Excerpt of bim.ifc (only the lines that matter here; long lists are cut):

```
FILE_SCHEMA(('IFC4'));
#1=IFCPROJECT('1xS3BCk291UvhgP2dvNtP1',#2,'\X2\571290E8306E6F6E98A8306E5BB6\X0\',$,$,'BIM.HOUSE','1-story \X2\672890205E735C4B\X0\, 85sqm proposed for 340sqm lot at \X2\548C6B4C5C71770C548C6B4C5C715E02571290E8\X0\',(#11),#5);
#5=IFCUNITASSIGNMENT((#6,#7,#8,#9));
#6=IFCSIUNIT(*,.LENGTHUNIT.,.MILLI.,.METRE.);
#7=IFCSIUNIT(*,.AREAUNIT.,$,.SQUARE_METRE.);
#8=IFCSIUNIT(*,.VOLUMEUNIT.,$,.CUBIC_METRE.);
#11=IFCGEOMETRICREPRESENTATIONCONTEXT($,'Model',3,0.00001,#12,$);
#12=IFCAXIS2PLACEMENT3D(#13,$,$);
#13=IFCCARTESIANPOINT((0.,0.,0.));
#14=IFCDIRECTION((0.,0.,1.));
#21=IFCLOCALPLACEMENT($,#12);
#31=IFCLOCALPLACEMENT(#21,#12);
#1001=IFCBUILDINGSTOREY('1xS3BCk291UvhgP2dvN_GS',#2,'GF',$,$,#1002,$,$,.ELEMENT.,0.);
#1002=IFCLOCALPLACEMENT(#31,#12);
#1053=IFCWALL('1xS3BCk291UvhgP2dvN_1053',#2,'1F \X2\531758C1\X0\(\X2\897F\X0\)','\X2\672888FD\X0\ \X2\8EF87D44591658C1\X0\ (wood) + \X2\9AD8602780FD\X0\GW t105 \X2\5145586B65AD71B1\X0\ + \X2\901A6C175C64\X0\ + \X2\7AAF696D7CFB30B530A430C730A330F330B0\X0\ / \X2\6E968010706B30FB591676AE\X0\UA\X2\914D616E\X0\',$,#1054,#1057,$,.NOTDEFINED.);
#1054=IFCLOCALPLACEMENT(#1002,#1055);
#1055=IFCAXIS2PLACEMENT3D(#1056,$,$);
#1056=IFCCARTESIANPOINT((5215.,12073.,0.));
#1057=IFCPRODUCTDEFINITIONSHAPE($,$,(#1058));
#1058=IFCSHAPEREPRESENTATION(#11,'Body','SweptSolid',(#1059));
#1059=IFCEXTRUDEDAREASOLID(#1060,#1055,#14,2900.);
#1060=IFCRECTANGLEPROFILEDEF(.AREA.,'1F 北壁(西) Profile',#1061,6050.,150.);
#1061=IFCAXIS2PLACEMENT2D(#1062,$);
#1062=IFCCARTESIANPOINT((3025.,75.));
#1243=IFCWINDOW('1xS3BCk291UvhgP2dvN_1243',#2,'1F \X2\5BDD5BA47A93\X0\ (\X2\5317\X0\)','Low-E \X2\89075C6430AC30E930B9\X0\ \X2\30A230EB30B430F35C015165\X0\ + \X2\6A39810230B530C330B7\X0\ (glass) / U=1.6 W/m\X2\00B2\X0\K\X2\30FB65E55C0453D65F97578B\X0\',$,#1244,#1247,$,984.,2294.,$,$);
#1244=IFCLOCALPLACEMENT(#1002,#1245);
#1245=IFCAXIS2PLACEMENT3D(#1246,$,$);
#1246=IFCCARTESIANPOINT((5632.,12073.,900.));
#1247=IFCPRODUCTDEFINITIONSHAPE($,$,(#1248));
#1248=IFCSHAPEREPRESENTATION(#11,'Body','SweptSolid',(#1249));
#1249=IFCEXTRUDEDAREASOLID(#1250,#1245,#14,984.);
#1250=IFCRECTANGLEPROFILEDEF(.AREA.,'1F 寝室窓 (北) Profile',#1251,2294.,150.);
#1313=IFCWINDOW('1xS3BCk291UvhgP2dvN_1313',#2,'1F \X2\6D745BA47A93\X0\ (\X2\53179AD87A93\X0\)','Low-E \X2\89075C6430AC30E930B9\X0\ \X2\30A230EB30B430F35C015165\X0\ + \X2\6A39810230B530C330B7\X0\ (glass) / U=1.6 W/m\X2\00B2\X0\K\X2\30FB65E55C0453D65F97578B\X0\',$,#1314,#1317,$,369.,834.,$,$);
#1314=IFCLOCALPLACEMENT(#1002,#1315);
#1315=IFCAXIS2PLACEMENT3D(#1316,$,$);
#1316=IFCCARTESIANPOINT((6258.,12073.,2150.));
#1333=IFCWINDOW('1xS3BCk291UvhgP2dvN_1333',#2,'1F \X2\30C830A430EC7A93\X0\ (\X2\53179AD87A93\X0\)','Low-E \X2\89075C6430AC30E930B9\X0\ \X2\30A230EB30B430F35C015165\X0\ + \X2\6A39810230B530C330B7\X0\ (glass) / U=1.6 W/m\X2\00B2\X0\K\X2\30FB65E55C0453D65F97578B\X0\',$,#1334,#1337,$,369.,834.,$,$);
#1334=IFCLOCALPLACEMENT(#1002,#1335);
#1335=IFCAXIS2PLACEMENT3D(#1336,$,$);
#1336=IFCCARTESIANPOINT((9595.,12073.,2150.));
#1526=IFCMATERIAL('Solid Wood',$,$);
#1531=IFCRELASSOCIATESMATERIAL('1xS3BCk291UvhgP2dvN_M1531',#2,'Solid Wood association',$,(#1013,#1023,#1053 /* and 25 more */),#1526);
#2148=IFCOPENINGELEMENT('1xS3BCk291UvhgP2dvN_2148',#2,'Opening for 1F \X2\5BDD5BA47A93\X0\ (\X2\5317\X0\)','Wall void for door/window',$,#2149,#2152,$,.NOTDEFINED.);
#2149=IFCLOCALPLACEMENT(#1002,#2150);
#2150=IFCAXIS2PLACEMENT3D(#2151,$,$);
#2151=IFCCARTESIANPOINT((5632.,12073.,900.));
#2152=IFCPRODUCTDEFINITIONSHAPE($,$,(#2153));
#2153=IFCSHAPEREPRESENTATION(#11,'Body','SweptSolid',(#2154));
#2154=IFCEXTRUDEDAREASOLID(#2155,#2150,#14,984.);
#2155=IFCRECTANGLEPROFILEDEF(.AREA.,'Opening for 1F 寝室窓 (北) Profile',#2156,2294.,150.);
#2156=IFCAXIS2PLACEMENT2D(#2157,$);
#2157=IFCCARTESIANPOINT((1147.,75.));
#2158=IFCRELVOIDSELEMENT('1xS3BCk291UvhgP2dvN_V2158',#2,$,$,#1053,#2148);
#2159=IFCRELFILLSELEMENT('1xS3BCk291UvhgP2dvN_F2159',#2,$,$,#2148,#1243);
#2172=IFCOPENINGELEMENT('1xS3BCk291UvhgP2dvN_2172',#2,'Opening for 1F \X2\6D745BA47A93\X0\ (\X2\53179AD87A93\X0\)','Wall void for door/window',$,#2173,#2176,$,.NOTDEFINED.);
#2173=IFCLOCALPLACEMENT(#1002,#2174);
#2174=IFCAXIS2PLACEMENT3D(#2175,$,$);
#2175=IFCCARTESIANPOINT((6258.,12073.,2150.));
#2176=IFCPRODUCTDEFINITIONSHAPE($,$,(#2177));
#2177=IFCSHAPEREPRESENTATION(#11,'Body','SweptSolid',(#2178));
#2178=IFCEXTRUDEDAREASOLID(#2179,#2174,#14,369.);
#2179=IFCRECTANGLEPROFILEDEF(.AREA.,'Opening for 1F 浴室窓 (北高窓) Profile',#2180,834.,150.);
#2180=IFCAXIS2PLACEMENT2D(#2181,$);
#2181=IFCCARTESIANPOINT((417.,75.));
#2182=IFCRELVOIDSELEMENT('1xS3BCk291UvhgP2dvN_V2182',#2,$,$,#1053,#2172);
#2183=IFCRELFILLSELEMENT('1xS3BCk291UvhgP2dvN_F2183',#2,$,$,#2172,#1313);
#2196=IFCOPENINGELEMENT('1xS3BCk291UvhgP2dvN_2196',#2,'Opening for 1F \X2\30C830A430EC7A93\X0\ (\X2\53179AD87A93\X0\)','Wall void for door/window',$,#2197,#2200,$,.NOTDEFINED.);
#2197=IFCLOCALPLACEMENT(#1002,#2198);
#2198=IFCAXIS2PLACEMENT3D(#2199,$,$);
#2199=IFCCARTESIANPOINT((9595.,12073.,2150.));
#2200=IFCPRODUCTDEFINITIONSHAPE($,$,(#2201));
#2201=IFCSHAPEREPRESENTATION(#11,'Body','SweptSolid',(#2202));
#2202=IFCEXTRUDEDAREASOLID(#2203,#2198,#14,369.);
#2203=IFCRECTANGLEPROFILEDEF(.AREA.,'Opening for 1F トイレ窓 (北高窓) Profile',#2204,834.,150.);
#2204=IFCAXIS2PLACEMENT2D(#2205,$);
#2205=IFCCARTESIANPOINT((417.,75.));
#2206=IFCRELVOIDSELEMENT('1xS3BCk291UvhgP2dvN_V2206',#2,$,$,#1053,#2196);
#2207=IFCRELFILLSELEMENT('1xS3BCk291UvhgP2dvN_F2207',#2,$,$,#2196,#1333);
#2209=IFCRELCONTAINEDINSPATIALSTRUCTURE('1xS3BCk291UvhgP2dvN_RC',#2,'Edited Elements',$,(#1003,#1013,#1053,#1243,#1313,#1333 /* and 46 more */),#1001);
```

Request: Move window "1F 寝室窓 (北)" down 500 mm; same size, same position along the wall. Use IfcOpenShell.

```python
import numpy as np
import ifcopenshell
import ifcopenshell.api.geometry
import ifcopenshell.util.placement
import ifcopenshell.util.unit

model = ifcopenshell.open("bim.ifc")
unit_scale = ifcopenshell.util.unit.calculate_unit_scale(model)

window = model.by_guid("1xS3BCk291UvhgP2dvN_1243")
opening = window.FillsVoids[0].RelatingOpeningElement
dz = -500.0

shift = np.array([0.0, 0.0, dz])
# The window is not placed relative to its opening, so move both.
for product in (opening, window):
    matrix = ifcopenshell.util.placement.get_local_placement(product.ObjectPlacement)
    matrix[:3, 3] += shift
    ifcopenshell.api.geometry.edit_object_placement(model, product=product, matrix=matrix, is_si=False)

print(f"moved by {dz * unit_scale:+.3f} m")

model.write("bim_rev.ifc")
```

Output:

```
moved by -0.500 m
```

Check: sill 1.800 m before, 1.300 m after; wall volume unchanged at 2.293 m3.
